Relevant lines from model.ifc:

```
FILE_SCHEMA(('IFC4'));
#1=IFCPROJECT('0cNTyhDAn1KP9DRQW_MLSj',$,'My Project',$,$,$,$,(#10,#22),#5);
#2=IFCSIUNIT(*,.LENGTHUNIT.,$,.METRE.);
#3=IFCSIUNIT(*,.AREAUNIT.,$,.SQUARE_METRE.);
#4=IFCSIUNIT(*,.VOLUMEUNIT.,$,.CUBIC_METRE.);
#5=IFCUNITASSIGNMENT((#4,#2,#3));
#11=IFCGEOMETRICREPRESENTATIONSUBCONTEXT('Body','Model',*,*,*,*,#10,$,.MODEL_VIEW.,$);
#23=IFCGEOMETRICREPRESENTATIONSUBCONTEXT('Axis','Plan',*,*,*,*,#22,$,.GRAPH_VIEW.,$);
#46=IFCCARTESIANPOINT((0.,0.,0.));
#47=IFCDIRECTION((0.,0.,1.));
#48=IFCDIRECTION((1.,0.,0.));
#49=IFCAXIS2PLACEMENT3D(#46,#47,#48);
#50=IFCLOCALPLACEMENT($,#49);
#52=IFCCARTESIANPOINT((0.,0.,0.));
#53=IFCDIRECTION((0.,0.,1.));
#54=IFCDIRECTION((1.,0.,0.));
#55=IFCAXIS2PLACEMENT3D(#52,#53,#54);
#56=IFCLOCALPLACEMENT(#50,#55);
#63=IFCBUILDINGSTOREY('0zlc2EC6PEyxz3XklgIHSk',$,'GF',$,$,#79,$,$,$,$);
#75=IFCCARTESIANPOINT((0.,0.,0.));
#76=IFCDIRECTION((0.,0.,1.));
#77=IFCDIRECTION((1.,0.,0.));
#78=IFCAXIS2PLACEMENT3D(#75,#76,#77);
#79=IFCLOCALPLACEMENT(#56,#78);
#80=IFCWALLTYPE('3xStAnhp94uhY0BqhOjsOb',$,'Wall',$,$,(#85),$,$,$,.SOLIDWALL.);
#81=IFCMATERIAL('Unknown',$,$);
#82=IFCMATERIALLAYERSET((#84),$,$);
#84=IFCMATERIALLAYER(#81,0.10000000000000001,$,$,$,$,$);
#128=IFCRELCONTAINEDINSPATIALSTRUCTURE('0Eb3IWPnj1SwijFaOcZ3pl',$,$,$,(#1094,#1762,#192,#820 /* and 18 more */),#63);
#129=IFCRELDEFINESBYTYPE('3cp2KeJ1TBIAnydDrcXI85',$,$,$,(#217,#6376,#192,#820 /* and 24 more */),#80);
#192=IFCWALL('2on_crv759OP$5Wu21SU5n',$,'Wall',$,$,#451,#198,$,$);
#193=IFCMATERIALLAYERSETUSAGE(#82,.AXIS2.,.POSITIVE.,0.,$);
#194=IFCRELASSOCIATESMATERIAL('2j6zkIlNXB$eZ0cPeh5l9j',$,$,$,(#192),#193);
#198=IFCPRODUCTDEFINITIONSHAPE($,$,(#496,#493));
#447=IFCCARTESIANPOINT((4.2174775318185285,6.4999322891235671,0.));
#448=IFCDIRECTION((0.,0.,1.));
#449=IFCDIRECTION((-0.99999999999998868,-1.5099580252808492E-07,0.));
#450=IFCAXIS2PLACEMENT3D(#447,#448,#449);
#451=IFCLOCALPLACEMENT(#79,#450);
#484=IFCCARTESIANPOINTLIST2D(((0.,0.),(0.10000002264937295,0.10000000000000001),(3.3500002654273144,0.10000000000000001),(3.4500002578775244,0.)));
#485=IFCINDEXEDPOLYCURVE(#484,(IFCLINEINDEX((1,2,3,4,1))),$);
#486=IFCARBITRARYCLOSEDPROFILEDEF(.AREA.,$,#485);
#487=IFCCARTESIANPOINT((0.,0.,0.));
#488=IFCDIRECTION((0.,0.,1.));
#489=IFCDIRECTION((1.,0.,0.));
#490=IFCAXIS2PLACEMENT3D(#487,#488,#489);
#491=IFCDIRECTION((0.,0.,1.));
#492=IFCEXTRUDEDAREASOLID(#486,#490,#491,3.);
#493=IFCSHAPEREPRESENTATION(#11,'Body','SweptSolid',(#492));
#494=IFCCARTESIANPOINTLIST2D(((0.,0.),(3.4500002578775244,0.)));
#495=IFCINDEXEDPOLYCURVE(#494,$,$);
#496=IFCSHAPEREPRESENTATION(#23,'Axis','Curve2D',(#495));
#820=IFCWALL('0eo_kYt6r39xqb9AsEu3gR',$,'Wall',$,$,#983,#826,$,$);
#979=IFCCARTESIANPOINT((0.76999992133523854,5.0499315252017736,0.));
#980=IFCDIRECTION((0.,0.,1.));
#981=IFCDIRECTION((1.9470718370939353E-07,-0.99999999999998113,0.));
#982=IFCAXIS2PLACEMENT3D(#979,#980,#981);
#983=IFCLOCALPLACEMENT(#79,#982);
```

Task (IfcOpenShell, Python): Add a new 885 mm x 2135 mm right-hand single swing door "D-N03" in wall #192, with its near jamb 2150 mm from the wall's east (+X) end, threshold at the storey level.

```python
import numpy as np
import ifcopenshell
import ifcopenshell.api.feature
import ifcopenshell.api.geometry
import ifcopenshell.api.root
import ifcopenshell.api.spatial
import ifcopenshell.geom
import ifcopenshell.util.element
import ifcopenshell.util.placement
import ifcopenshell.util.representation
import ifcopenshell.util.shape
import ifcopenshell.util.unit

model = ifcopenshell.open("model.ifc")
unit_scale = ifcopenshell.util.unit.calculate_unit_scale(model)
settings = ifcopenshell.geom.settings()


def volume(element):
    """Net volume in cubic metres, openings subtracted."""
    shape = ifcopenshell.geom.create_shape(settings, element)
    return ifcopenshell.util.shape.get_volume(shape.geometry)


wall = model.by_guid("2on_crv759OP$5Wu21SU5n")
storey = ifcopenshell.util.element.get_container(wall, ifc_class="IfcBuildingStorey")
context = ifcopenshell.util.representation.get_context(model, "Model", "Body", "MODEL_VIEW")
before = volume(wall)

width, height, from_end, sill = 0.885, 2.135, 2.15, 0.0  # metres

# The wall runs along its own X axis, and the end named is its -X end.
wall_shape = ifcopenshell.geom.create_shape(settings, wall)
x, y, z = ifcopenshell.util.shape.get_vertices(wall_shape.geometry).T
start = x.min() + from_end
face, thickness = float(y.min()), float(y.max() - y.min())
wall_matrix = ifcopenshell.util.placement.get_local_placement(wall.ObjectPlacement)
level = ifcopenshell.util.placement.get_local_placement(storey.ObjectPlacement)[2, 3]


def in_wall(x, y):
    """Placement at x, y metres in the wall's axes, at sill height."""
    matrix = wall_matrix.copy()
    matrix[:, 3] = wall_matrix @ np.array([x / unit_scale, y / unit_scale, 0.0, 1.0])
    matrix[2, 3] = level + sill / unit_scale
    return matrix


# Opening: a box that overshoots both wall faces by 50 mm.
opening = ifcopenshell.api.root.create_entity(model, ifc_class="IfcOpeningElement", predefined_type="OPENING")
box = ifcopenshell.api.geometry.add_wall_representation(
    model, context=context, length=width, height=height, thickness=thickness + 0.1
)
ifcopenshell.api.geometry.assign_representation(model, product=opening, representation=box)
ifcopenshell.api.geometry.edit_object_placement(model, product=opening, matrix=in_wall(start, face - 0.05), is_si=False)
ifcopenshell.api.feature.add_feature(model, feature=opening, element=wall)

door = ifcopenshell.api.root.create_entity(model, ifc_class="IfcDoor", name="D-N03", predefined_type="DOOR")
door.OverallWidth, door.OverallHeight = width / unit_scale, height / unit_scale
door.OperationType = "SINGLE_SWING_RIGHT"
body = ifcopenshell.api.geometry.add_door_representation(
    model,
    context=context,
    overall_width=door.OverallWidth,
    overall_height=door.OverallHeight,
    operation_type="SINGLE_SWING_RIGHT",
    lining_properties={"LiningDepth": thickness / unit_scale, "ThresholdDepth": thickness / unit_scale},
)
ifcopenshell.api.geometry.assign_representation(model, product=door, representation=body)
ifcopenshell.api.spatial.assign_container(model, products=[door], relating_structure=storey)
ifcopenshell.api.feature.add_filling(model, opening=opening, element=door)

# The lining spans the wall, so the door starts at the wall face.
ifcopenshell.api.geometry.edit_object_placement(model, product=door, matrix=in_wall(start, face), is_si=False)

after = volume(wall)

print(f"wall volume {before:.3f} -> {after:.3f} m3")

model.write("model_v2.ifc")
```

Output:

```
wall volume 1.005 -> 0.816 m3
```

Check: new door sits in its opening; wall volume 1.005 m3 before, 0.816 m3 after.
